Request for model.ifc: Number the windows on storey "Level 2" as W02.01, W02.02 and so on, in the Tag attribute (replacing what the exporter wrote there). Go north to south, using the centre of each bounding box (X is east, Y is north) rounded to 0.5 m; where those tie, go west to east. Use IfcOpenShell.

First a look at what the model holds.

```python
import ifcopenshell
import ifcopenshell.util.element
import ifcopenshell.util.placement

model = ifcopenshell.open("model.ifc")
print(model.schema)
storey = next(s for s in model.by_type("IfcBuildingStorey") if s.Name == "Level 2")
windows = [e for e in ifcopenshell.util.element.get_decomposition(storey) if e.is_a("IfcWindow")]
for e in sorted(windows, key=lambda e: e.id()):
    origin = ifcopenshell.util.placement.get_local_placement(e.ObjectPlacement)[:3, 3]
    print(e.id(), e.Tag, e.Name, origin.round(2) + 0.0, sep=" | ")
```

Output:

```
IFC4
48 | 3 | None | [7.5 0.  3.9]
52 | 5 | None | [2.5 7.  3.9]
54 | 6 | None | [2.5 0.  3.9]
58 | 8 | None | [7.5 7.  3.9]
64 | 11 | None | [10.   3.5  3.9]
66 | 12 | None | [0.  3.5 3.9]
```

```python
import ifcopenshell
import ifcopenshell.geom
import ifcopenshell.util.element
import ifcopenshell.util.shape

model = ifcopenshell.open("model.ifc")
settings = ifcopenshell.geom.settings()
settings.set("use-world-coords", True)


def centre(element):
    shape = ifcopenshell.geom.create_shape(settings, element)
    return ifcopenshell.util.shape.get_bbox_centroid(shape.geometry)


storey = next(s for s in model.by_type("IfcBuildingStorey") if s.Name == "Level 2")
windows = [e for e in ifcopenshell.util.element.get_decomposition(storey) if e.is_a("IfcWindow")]

# Insertion points can sit at a corner or the storey origin, so sort by the geometry (in metres).
centres = {e: centre(e) for e in windows}
windows.sort(key=lambda e: (-round(centres[e][1] / 0.5), centres[e][0]))

for i, e in enumerate(windows, start=1):
    number = f"W02.{i:02d}"
    e.Tag = number
    print(e.id(), number)

model.write("model_updated.ifc")
```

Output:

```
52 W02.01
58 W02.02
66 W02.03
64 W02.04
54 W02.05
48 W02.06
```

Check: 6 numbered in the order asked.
